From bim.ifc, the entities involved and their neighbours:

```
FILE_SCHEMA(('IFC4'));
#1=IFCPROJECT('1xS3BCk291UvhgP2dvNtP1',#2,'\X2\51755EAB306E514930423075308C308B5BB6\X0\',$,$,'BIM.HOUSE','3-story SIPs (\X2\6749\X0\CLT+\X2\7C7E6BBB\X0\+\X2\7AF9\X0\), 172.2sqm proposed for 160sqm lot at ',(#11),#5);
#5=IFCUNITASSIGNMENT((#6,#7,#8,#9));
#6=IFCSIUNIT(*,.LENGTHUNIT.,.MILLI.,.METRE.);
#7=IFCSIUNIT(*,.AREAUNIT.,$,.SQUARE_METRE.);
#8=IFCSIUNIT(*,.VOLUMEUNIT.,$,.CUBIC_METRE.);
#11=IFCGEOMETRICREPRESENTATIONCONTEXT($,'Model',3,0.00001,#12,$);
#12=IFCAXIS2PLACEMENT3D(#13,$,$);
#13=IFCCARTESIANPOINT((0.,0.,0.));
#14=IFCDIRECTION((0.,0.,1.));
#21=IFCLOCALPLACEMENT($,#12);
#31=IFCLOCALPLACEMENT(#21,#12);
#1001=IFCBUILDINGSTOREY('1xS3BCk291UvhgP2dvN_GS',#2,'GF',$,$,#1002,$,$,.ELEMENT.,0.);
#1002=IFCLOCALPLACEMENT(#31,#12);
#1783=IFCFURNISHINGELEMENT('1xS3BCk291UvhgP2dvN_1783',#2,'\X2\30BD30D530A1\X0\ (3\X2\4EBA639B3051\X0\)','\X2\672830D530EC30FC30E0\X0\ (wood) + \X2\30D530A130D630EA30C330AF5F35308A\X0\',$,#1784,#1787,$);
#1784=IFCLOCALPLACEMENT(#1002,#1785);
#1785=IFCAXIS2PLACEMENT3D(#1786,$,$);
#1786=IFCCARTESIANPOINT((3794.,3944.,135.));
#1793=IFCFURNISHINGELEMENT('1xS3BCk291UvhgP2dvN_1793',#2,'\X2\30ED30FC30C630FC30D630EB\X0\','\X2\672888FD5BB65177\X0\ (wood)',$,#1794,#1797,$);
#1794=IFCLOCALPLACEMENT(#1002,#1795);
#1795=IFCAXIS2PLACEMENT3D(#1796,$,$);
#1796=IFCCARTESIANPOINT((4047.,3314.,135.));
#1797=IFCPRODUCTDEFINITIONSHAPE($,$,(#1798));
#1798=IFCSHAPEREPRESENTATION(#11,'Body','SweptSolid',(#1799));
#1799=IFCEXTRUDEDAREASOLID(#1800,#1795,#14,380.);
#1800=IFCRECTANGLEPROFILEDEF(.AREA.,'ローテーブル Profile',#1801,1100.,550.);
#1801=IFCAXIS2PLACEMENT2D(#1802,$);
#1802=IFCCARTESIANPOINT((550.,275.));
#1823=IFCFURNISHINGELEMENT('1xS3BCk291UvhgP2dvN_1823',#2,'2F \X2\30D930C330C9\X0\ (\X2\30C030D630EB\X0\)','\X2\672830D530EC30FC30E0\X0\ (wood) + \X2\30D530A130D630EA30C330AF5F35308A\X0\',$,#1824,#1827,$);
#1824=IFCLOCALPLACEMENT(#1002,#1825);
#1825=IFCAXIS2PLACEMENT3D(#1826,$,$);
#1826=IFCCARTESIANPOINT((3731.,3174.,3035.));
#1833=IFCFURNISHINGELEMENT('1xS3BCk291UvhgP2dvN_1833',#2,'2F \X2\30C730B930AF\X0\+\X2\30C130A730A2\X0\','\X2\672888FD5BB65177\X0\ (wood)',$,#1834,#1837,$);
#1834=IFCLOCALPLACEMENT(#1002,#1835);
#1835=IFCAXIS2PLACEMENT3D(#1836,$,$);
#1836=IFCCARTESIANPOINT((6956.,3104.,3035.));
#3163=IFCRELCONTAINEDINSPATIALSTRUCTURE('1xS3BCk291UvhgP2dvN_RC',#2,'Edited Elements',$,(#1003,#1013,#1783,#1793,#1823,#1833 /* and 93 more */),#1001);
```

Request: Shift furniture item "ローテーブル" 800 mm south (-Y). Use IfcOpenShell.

```python
import ifcopenshell
import ifcopenshell.api.geometry
import ifcopenshell.util.placement

model = ifcopenshell.open("bim.ifc")

item = model.by_guid("1xS3BCk291UvhgP2dvN_1793")
matrix = ifcopenshell.util.placement.get_local_placement(item.ObjectPlacement)
matrix[1, 3] -= 800.0
ifcopenshell.api.geometry.edit_object_placement(model, product=item, matrix=matrix, is_si=False)

print(ifcopenshell.util.placement.get_local_placement(item.ObjectPlacement).round(3) + 0.0)

model.write("bim_edited.ifc")
```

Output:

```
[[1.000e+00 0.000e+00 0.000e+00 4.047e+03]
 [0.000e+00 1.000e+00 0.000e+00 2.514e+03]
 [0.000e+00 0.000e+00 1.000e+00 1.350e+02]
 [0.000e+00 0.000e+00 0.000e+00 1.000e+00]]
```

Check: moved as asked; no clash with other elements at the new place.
